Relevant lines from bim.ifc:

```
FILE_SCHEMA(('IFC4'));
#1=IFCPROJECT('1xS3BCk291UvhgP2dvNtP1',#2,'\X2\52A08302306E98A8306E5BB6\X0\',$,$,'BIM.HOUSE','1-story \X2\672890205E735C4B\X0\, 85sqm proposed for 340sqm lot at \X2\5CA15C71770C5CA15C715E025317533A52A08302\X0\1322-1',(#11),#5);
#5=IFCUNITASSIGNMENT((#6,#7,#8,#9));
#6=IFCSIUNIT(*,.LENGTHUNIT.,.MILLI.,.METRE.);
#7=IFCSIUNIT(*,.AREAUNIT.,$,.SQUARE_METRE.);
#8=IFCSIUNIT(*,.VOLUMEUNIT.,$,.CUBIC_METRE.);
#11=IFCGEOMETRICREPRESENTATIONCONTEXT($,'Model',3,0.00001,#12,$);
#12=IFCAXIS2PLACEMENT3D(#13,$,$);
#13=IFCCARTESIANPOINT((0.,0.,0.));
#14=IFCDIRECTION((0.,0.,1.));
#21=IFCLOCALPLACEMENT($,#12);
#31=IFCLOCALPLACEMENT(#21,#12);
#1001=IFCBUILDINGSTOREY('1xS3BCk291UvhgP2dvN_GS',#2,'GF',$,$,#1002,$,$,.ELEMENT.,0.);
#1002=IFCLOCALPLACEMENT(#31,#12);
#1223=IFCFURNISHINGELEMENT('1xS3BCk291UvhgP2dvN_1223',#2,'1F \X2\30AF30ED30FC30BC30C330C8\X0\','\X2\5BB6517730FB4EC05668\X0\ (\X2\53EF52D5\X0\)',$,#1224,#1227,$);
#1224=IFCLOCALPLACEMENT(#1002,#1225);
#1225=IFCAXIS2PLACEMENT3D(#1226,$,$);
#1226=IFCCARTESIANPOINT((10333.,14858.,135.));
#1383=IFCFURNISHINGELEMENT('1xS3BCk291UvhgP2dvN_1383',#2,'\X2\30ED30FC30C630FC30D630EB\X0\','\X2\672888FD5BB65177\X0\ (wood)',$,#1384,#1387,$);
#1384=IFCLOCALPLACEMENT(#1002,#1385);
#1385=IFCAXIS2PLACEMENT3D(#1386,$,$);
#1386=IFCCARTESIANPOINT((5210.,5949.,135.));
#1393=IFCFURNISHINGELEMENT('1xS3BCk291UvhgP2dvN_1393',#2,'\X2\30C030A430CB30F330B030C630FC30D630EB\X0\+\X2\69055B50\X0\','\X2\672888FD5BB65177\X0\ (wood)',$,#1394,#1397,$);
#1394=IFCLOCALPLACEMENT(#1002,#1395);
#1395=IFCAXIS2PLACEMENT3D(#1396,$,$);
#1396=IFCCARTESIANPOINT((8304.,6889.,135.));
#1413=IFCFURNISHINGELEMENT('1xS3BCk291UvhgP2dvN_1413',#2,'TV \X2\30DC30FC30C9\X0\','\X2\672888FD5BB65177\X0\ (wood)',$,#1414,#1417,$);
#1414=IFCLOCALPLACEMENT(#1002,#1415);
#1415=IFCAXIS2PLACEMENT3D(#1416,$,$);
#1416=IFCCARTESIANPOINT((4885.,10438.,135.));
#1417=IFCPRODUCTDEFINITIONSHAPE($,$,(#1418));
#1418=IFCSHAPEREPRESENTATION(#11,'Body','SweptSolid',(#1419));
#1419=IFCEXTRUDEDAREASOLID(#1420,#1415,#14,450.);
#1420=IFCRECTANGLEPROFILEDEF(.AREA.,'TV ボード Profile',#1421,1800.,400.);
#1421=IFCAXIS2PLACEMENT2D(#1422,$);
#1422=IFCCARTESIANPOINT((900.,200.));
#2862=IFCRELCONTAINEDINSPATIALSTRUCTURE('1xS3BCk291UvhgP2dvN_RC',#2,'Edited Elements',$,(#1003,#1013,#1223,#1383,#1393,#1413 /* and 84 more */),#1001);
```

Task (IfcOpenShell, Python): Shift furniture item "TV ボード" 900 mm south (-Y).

```python
import ifcopenshell
import ifcopenshell.api.geometry
import ifcopenshell.util.placement
import ifcopenshell.util.unit

model = ifcopenshell.open("bim.ifc")
unit_scale = ifcopenshell.util.unit.calculate_unit_scale(model)

item = model.by_guid("1xS3BCk291UvhgP2dvN_1413")
matrix = ifcopenshell.util.placement.get_local_placement(item.ObjectPlacement)
matrix[1, 3] -= 0.9 / unit_scale
ifcopenshell.api.geometry.edit_object_placement(model, product=item, matrix=matrix, is_si=False)

print(ifcopenshell.util.placement.get_local_placement(item.ObjectPlacement).round(3) + 0.0)

model.write("bim-out.ifc")
```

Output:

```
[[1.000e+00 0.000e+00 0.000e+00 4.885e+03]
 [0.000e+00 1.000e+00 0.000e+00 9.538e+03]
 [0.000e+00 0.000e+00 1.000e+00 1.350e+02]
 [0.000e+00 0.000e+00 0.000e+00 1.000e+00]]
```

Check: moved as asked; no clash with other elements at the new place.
